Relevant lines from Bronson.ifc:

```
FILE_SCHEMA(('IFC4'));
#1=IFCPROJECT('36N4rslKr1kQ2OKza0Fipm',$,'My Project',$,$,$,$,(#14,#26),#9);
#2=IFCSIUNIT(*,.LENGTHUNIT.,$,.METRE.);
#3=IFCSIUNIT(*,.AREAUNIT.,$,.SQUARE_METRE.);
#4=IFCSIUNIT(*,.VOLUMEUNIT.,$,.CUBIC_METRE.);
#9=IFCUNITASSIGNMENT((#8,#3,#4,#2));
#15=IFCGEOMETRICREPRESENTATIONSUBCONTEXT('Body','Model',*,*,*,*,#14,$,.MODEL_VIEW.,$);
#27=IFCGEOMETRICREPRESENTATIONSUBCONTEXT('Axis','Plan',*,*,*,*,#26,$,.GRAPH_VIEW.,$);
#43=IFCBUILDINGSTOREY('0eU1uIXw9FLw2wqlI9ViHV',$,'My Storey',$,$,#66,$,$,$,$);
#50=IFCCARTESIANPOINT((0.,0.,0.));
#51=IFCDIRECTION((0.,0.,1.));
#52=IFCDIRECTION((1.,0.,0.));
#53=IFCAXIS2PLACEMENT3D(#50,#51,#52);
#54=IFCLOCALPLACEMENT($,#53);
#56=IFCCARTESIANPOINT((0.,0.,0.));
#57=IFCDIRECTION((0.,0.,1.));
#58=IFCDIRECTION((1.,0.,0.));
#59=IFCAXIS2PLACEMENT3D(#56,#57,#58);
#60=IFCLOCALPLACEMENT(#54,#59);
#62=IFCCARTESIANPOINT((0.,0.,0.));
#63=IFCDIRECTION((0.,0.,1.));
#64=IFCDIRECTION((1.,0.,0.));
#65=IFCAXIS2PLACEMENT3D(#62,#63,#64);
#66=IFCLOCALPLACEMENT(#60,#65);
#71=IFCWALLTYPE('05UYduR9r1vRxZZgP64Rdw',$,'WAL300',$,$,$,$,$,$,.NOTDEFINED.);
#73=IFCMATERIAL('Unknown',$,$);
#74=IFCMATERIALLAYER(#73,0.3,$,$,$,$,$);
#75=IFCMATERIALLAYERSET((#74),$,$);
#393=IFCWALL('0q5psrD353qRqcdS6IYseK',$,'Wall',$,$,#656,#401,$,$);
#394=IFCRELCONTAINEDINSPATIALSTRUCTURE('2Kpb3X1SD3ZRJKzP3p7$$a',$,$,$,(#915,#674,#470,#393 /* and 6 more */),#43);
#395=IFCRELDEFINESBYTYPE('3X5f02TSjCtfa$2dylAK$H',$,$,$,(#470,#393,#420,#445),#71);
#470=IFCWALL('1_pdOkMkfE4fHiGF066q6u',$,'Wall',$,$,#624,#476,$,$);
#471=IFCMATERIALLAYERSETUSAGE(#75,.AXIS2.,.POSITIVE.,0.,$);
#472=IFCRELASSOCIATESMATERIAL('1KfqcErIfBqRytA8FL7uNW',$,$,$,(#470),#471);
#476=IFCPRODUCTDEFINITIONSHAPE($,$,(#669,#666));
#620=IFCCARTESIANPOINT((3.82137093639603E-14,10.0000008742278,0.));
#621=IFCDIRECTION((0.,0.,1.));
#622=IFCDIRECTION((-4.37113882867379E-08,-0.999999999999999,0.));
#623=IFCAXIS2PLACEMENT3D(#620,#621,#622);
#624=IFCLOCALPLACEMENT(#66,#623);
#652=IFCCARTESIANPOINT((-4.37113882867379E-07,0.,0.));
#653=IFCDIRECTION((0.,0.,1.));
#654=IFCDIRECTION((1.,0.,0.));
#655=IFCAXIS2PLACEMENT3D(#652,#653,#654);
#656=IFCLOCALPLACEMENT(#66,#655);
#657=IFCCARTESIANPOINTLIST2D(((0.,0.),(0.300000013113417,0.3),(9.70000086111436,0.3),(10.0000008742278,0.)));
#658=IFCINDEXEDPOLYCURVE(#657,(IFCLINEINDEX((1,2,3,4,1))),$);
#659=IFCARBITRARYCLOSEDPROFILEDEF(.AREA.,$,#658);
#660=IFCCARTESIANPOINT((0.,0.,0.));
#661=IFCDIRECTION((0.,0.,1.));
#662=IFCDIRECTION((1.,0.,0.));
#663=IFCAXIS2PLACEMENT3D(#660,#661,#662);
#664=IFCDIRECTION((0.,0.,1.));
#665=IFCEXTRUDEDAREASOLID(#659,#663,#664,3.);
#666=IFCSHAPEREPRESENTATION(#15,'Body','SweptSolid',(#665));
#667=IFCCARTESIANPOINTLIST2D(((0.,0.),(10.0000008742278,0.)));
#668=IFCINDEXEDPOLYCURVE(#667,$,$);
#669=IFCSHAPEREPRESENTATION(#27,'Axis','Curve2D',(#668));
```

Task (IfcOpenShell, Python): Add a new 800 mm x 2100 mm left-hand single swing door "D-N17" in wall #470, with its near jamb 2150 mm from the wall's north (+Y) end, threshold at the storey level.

```python
import numpy as np
import ifcopenshell
import ifcopenshell.api.feature
import ifcopenshell.api.geometry
import ifcopenshell.api.root
import ifcopenshell.api.spatial
import ifcopenshell.geom
import ifcopenshell.util.element
import ifcopenshell.util.placement
import ifcopenshell.util.representation
import ifcopenshell.util.shape
import ifcopenshell.util.unit

model = ifcopenshell.open("Bronson.ifc")
unit_scale = ifcopenshell.util.unit.calculate_unit_scale(model)
settings = ifcopenshell.geom.settings()


def volume(element):
    """Net volume in cubic metres, openings subtracted."""
    shape = ifcopenshell.geom.create_shape(settings, element)
    return ifcopenshell.util.shape.get_volume(shape.geometry)


wall = model.by_id(470)
storey = ifcopenshell.util.element.get_container(wall, ifc_class="IfcBuildingStorey")
context = ifcopenshell.util.representation.get_context(model, "Model", "Body", "MODEL_VIEW")
before = volume(wall)

width, height, from_end, sill = 0.8, 2.1, 2.15, 0.0  # metres

# The wall runs along its own X axis, and the end named is its -X end.
wall_shape = ifcopenshell.geom.create_shape(settings, wall)
x, y, z = ifcopenshell.util.shape.get_vertices(wall_shape.geometry).T
start = x.min() + from_end
face, thickness = float(y.min()), float(y.max() - y.min())
wall_matrix = ifcopenshell.util.placement.get_local_placement(wall.ObjectPlacement)
level = ifcopenshell.util.placement.get_local_placement(storey.ObjectPlacement)[2, 3]


def in_wall(x, y):
    """Placement at x, y metres in the wall's axes, at sill height."""
    matrix = wall_matrix.copy()
    matrix[:, 3] = wall_matrix @ np.array([x / unit_scale, y / unit_scale, 0.0, 1.0])
    matrix[2, 3] = level + sill / unit_scale
    return matrix


# Opening: a box that overshoots both wall faces by 50 mm.
opening = ifcopenshell.api.root.create_entity(model, ifc_class="IfcOpeningElement", predefined_type="OPENING")
box = ifcopenshell.api.geometry.add_wall_representation(
    model, context=context, length=width, height=height, thickness=thickness + 0.1
)
ifcopenshell.api.geometry.assign_representation(model, product=opening, representation=box)
ifcopenshell.api.geometry.edit_object_placement(model, product=opening, matrix=in_wall(start, face - 0.05), is_si=False)
ifcopenshell.api.feature.add_feature(model, feature=opening, element=wall)

door = ifcopenshell.api.root.create_entity(model, ifc_class="IfcDoor", name="D-N17", predefined_type="DOOR")
door.OverallWidth, door.OverallHeight = width / unit_scale, height / unit_scale
door.OperationType = "SINGLE_SWING_LEFT"
body = ifcopenshell.api.geometry.add_door_representation(
    model,
    context=context,
    overall_width=door.OverallWidth,
    overall_height=door.OverallHeight,
    operation_type="SINGLE_SWING_LEFT",
    lining_properties={"LiningDepth": thickness / unit_scale, "ThresholdDepth": thickness / unit_scale},
)
ifcopenshell.api.geometry.assign_representation(model, product=door, representation=body)
ifcopenshell.api.spatial.assign_container(model, products=[door], relating_structure=storey)
ifcopenshell.api.feature.add_filling(model, opening=opening, element=door)

# The lining spans the wall, so the door starts at the wall face.
ifcopenshell.api.geometry.edit_object_placement(model, product=door, matrix=in_wall(start, face), is_si=False)

after = volume(wall)

print(f"wall volume {before:.3f} -> {after:.3f} m3")

model.write("Bronson_edited.ifc")
```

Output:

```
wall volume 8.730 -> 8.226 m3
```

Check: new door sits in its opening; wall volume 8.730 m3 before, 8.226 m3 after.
